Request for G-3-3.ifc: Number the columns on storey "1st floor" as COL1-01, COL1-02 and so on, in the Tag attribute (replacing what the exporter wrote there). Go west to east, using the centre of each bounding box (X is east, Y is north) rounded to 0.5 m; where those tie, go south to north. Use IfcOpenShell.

First a look at what the model holds.

```python
import ifcopenshell
import ifcopenshell.util.element
import ifcopenshell.util.placement

model = ifcopenshell.open("G-3-3.ifc")
print(model.schema)
storey = next(s for s in model.by_type("IfcBuildingStorey") if s.Name == "1st floor")
columns = [e for e in ifcopenshell.util.element.get_decomposition(storey) if e.is_a("IfcColumn")]
for e in sorted(columns, key=lambda e: e.id()):
    origin = ifcopenshell.util.placement.get_local_placement(e.ObjectPlacement)[:3, 3]
    print(e.id(), e.Tag, e.Name, origin.round(2) + 0.0, sep=" | ")
```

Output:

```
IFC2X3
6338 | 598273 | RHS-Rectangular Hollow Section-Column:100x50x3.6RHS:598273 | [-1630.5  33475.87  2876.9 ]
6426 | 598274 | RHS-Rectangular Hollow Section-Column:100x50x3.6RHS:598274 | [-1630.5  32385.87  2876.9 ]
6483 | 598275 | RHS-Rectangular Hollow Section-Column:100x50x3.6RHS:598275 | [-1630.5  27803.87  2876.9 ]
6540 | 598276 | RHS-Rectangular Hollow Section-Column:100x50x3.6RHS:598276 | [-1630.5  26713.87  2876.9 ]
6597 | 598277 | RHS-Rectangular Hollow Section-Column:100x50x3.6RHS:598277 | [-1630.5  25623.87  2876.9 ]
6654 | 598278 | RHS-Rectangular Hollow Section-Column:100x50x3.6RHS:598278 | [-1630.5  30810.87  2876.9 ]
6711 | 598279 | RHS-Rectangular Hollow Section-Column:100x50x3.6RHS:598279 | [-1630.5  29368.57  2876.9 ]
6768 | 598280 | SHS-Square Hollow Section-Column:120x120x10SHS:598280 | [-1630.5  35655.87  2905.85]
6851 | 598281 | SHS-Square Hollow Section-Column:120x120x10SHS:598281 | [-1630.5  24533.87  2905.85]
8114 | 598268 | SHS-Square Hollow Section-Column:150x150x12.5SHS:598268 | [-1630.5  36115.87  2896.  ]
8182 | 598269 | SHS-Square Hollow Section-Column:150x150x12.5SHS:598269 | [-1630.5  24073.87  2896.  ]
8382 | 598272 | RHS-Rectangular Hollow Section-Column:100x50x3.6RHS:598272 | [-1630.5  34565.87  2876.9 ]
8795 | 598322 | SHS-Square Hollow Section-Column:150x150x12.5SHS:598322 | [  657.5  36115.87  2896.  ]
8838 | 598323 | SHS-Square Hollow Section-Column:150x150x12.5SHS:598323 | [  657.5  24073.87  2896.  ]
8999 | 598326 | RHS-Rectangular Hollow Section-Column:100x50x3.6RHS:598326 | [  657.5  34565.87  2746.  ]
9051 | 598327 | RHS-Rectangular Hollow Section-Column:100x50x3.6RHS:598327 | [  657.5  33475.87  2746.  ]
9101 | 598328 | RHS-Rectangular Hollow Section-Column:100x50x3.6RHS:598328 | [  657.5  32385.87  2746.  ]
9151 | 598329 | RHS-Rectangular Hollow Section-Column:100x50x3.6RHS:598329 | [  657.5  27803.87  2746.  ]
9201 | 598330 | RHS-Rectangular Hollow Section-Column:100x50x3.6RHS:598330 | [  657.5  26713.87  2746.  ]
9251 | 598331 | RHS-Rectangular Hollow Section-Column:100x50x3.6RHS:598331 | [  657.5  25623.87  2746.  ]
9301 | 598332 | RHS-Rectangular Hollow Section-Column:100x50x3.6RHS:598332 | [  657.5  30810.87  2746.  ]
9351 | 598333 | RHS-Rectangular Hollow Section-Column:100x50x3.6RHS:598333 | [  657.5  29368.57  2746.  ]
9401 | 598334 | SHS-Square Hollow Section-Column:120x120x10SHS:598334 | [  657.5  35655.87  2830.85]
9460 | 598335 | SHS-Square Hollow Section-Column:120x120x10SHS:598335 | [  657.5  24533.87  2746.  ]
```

```python
import ifcopenshell
import ifcopenshell.geom
import ifcopenshell.util.element
import ifcopenshell.util.shape

model = ifcopenshell.open("G-3-3.ifc")
settings = ifcopenshell.geom.settings()
settings.set("use-world-coords", True)


def centre(element):
    shape = ifcopenshell.geom.create_shape(settings, element)
    return ifcopenshell.util.shape.get_bbox_centroid(shape.geometry)


storey = next(s for s in model.by_type("IfcBuildingStorey") if s.Name == "1st floor")
columns = [e for e in ifcopenshell.util.element.get_decomposition(storey) if e.is_a("IfcColumn")]

# Insertion points can sit at a corner or the storey origin, so sort by the geometry (in metres).
centres = {e: centre(e) for e in columns}
columns.sort(key=lambda e: (round(centres[e][0] / 0.5), centres[e][1]))

for i, e in enumerate(columns, start=1):
    number = f"COL1-{i:02d}"
    e.Tag = number
    print(e.id(), number)

model.write("G-3-3_rev.ifc")
```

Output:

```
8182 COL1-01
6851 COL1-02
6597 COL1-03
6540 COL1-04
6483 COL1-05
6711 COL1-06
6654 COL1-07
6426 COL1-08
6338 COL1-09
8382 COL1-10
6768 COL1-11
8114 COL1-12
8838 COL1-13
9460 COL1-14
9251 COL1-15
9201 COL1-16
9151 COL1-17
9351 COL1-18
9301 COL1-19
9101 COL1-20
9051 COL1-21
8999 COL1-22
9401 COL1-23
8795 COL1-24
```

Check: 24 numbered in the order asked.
